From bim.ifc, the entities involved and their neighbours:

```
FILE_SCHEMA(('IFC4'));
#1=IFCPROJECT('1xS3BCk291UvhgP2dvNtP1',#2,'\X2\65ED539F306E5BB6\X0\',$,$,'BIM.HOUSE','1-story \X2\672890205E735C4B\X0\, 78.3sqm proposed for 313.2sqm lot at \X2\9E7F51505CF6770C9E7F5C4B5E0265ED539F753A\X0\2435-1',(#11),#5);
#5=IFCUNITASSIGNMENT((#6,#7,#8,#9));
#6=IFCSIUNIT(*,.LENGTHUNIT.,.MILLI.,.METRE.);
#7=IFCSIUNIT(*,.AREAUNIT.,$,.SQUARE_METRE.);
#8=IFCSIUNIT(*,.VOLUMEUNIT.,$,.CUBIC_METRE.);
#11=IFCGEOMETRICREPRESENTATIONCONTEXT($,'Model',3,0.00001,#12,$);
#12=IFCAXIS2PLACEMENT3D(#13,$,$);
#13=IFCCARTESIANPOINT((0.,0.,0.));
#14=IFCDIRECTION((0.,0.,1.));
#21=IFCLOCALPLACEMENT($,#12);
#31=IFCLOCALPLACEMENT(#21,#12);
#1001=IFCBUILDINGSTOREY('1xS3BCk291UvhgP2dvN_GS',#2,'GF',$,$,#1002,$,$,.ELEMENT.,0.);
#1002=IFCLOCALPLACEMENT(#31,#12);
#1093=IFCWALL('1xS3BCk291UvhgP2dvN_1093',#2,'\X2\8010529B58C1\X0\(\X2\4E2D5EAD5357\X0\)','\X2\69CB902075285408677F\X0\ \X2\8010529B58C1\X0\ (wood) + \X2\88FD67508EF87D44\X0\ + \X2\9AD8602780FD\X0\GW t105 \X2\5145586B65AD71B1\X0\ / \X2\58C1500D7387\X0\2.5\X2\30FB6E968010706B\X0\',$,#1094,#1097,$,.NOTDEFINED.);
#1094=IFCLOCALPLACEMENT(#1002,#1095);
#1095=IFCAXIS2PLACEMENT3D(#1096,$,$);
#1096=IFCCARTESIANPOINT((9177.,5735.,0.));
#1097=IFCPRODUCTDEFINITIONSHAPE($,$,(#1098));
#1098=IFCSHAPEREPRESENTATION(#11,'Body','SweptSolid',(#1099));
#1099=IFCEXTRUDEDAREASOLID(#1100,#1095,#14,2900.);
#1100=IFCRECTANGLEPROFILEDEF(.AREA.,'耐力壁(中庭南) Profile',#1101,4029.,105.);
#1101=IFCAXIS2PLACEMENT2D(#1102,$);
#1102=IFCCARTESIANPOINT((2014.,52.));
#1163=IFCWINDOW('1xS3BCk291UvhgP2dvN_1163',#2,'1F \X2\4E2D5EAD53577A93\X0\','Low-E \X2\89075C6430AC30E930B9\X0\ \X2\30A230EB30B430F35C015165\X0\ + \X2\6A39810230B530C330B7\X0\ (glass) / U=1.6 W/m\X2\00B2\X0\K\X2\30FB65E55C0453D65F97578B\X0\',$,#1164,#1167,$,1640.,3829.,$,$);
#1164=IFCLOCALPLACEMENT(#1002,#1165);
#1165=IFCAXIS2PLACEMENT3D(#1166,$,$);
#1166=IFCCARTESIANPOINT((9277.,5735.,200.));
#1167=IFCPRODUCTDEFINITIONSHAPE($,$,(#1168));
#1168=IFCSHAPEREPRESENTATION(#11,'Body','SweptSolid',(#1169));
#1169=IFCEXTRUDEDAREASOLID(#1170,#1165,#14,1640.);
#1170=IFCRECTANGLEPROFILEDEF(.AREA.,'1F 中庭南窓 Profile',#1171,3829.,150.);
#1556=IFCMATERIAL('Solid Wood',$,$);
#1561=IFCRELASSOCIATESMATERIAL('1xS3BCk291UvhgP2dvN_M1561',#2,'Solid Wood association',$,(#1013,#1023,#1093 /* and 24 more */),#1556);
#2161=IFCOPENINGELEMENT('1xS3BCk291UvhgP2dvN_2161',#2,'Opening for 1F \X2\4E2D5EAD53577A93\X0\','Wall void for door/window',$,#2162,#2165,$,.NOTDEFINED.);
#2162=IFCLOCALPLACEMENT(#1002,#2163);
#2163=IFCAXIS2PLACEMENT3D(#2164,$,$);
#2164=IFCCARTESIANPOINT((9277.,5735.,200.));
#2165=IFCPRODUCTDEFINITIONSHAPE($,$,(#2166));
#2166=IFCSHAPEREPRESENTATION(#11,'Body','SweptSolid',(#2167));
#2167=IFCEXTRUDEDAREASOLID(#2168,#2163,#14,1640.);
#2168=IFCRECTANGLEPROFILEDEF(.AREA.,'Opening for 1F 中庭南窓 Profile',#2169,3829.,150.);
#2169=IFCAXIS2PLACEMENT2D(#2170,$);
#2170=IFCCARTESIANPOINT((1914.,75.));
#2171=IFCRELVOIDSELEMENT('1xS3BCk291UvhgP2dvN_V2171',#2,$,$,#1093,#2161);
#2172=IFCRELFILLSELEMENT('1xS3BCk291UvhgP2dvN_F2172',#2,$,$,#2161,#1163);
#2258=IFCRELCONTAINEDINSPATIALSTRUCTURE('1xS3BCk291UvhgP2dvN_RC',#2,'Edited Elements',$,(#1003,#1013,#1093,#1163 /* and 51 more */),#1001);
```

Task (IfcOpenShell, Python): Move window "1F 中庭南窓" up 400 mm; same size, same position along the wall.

```python
import numpy as np
import ifcopenshell
import ifcopenshell.api.geometry
import ifcopenshell.util.placement
import ifcopenshell.util.unit

model = ifcopenshell.open("bim.ifc")
unit_scale = ifcopenshell.util.unit.calculate_unit_scale(model)

window = model.by_guid("1xS3BCk291UvhgP2dvN_1163")
opening = window.FillsVoids[0].RelatingOpeningElement
dz = 400.0

shift = np.array([0.0, 0.0, dz])
# The window is not placed relative to its opening, so move both.
for product in (opening, window):
    matrix = ifcopenshell.util.placement.get_local_placement(product.ObjectPlacement)
    matrix[:3, 3] += shift
    ifcopenshell.api.geometry.edit_object_placement(model, product=product, matrix=matrix, is_si=False)

print(f"moved by {dz * unit_scale:+.3f} m")

model.write("bim_rev.ifc")
```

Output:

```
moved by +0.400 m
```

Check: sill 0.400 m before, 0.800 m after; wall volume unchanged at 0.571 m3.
